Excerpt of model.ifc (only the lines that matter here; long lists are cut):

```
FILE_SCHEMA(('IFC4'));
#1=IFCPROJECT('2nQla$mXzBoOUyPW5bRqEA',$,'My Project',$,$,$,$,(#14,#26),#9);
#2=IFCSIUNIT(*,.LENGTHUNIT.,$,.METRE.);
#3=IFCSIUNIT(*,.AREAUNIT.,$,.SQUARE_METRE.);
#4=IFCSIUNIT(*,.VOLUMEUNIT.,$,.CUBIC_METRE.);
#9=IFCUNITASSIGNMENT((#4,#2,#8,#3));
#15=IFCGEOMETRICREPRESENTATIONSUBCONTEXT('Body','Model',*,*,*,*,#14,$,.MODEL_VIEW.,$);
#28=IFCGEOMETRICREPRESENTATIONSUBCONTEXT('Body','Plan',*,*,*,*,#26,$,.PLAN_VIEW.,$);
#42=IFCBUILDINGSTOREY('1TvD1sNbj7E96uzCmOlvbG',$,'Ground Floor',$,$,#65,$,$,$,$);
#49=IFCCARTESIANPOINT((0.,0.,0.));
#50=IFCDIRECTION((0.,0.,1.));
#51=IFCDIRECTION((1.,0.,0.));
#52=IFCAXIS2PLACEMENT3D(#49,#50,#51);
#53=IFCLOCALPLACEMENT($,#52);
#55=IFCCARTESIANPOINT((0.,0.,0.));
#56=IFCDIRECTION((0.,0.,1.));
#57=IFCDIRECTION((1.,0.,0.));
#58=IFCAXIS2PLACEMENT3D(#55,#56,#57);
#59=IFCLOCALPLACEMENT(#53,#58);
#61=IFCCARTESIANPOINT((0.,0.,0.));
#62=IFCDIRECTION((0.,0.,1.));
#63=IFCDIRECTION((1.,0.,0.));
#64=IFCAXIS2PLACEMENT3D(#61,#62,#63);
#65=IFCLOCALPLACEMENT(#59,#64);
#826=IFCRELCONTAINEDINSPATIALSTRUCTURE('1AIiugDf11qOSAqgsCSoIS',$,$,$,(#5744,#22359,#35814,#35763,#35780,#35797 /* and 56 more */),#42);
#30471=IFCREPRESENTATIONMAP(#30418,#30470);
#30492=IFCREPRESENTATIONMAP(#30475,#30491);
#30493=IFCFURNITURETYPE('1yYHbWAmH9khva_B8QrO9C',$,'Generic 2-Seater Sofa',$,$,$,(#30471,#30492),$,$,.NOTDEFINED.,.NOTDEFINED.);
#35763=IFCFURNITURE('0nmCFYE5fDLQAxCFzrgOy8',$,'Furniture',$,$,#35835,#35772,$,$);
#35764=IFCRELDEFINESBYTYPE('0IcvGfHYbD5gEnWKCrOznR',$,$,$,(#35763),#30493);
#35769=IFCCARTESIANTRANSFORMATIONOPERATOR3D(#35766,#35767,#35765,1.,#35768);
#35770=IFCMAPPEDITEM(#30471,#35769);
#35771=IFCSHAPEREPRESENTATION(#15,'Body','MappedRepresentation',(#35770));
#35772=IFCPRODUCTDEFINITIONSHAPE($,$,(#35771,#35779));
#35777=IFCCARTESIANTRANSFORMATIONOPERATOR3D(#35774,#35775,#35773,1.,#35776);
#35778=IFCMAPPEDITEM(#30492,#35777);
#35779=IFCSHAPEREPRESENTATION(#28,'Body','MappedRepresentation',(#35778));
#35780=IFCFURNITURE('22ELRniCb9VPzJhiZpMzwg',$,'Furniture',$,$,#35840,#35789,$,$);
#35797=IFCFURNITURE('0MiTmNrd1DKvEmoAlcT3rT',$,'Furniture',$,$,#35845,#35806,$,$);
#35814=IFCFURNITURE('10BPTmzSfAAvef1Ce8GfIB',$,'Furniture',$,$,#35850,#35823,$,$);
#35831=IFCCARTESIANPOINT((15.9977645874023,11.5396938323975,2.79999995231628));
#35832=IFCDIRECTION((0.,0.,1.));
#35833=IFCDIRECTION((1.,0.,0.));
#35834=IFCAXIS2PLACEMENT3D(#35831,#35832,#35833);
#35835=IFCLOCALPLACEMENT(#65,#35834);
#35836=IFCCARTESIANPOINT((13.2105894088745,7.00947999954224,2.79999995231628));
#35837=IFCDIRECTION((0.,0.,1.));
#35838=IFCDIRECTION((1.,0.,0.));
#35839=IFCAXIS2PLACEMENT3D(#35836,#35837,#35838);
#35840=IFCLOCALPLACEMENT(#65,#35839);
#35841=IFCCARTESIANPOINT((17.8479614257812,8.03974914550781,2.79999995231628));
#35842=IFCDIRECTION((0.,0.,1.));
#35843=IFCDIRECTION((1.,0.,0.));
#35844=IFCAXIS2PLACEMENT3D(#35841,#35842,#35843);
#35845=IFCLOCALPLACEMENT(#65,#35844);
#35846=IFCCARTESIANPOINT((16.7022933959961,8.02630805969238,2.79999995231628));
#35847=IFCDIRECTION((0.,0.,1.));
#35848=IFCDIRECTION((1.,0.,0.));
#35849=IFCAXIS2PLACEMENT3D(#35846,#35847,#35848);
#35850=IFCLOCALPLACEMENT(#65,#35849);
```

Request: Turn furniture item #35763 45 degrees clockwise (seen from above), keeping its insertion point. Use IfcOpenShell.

```python
import ifcopenshell
import ifcopenshell.api.geometry
import ifcopenshell.util.placement

model = ifcopenshell.open("model.ifc")

item = model.by_guid("0nmCFYE5fDLQAxCFzrgOy8")
matrix = ifcopenshell.util.placement.get_local_placement(item.ObjectPlacement)
matrix = matrix @ ifcopenshell.util.placement.rotation(-45, "Z")
ifcopenshell.api.geometry.edit_object_placement(model, product=item, matrix=matrix, is_si=False)

print(ifcopenshell.util.placement.get_local_placement(item.ObjectPlacement).round(3) + 0.0)

model.write("model-out.ifc")
```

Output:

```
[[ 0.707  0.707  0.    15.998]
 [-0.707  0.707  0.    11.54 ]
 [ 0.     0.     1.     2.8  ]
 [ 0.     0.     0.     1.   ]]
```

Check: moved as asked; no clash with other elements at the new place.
